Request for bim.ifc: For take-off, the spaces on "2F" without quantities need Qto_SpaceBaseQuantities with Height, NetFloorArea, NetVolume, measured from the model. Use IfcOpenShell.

First a look at what the model holds.

```python
import ifcopenshell
import ifcopenshell.util.element
import ifcopenshell.util.unit

model = ifcopenshell.open("bim.ifc")
print(model.schema)
for unit_type in ("LENGTHUNIT", "AREAUNIT", "VOLUMEUNIT"):
    print(unit_type, ifcopenshell.util.unit.calculate_unit_scale(model, unit_type))
storey = next(s for s in model.by_type("IfcBuildingStorey") if s.Name == "2F")
spaces = [e for e in ifcopenshell.util.element.get_decomposition(storey) if e.is_a("IfcSpace")]
for e in sorted(spaces, key=lambda e: e.id()):
    print(e.id(), e.is_a(), e.Name, list(ifcopenshell.util.element.get_psets(e, qtos_only=True)), sep=" | ")
```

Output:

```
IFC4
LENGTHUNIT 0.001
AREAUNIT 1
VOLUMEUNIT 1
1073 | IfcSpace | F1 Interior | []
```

```python
import ifcopenshell
import ifcopenshell.api.pset
import ifcopenshell.geom
import ifcopenshell.util.element
import ifcopenshell.util.shape
import ifcopenshell.util.unit

model = ifcopenshell.open("bim.ifc")
unit_scale = ifcopenshell.util.unit.calculate_unit_scale(model)
area_scale = ifcopenshell.util.unit.calculate_unit_scale(model, "AREAUNIT")
volume_scale = ifcopenshell.util.unit.calculate_unit_scale(model, "VOLUMEUNIT")
settings = ifcopenshell.geom.settings()

storey = next(s for s in model.by_type("IfcBuildingStorey") if s.Name == "2F")
spaces = [e for e in ifcopenshell.util.element.get_decomposition(storey) if e.is_a("IfcSpace")]

for e in sorted(spaces, key=lambda e: e.id()):
    if ifcopenshell.util.element.get_psets(e, qtos_only=True, should_inherit=False):
        continue
    # Geometry comes back in metres, in the element's own axes.
    shape = ifcopenshell.geom.create_shape(settings, e)
    values = {
        "Height": ifcopenshell.util.shape.get_z(shape.geometry) / unit_scale,
        "NetFloorArea": ifcopenshell.util.shape.get_footprint_area(shape.geometry) / area_scale,
        "NetVolume": ifcopenshell.util.shape.get_volume(shape.geometry) / volume_scale,
    }
    qto = ifcopenshell.api.pset.add_qto(model, product=e, name="Qto_SpaceBaseQuantities")
    ifcopenshell.api.pset.edit_qto(model, qto=qto, properties=values)
    print(e.id(), {k: round(v, 3) for k, v in values.items()})

model.write("bim_v2.ifc")
```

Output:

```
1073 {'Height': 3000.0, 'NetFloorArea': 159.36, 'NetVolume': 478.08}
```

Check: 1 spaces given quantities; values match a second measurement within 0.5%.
